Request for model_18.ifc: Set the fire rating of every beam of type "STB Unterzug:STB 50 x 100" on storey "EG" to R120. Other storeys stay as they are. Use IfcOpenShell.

First a look at what the model holds.

```python
import ifcopenshell
import ifcopenshell.util.element

model = ifcopenshell.open("model_18.ifc")
print(model.schema)
storey = next(s for s in model.by_type("IfcBuildingStorey") if s.Name == "EG")
beams = [e for e in ifcopenshell.util.element.get_decomposition(storey) if e.is_a("IfcBeam")]
seen = {}
for e in beams:
    element_type = ifcopenshell.util.element.get_type(e)
    key = (element_type.Name if element_type != e and element_type else None, ifcopenshell.util.element.get_pset(e, "Pset_BeamCommon", "FireRating"))
    seen[key] = seen.get(key, 0) + 1
for (name, value), count in sorted(seen.items(), key=str):
    print(count, "x", name, "|", value)
```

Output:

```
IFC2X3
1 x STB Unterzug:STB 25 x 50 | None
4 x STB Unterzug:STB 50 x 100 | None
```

```python
import ifcopenshell
import ifcopenshell.api.pset
import ifcopenshell.util.element

model = ifcopenshell.open("model_18.ifc")

storey = next(s for s in model.by_type("IfcBuildingStorey") if s.Name == "EG")
beams = [e for e in ifcopenshell.util.element.get_decomposition(storey) if e.is_a("IfcBeam")]

count = 0
for e in beams:
    element_type = ifcopenshell.util.element.get_type(e)
    if element_type in (None, e) or element_type.Name != "STB Unterzug:STB 50 x 100":
        continue
    # add_pset returns the element's existing set when there is one.
    pset = ifcopenshell.api.pset.add_pset(model, product=e, name="Pset_BeamCommon")
    ifcopenshell.api.pset.edit_pset(model, pset=pset, properties={"FireRating": "R120"})
    count += 1

print(count, "beams updated")

model.write("model_18_updated.ifc")
```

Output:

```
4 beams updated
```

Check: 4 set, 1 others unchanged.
